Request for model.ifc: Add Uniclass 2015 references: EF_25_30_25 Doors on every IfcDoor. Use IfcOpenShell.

First a look at what the model holds.

```python
import ifcopenshell

model = ifcopenshell.open("model.ifc")
print(model.schema)
print("classifications:", [c.Name for c in model.by_type("IfcClassification")])
for ifc_class in ("IfcDoor", "IfcRoof", "IfcStair", "IfcWall", "IfcWindow"):
    print(ifc_class, len(model.by_type(ifc_class)))
```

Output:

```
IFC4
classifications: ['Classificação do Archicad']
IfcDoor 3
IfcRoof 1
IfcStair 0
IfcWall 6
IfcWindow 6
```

```python
import ifcopenshell
import ifcopenshell.api.classification

model = ifcopenshell.open("model.ifc")

system = ifcopenshell.api.classification.add_classification(model, classification="Uniclass 2015")

codes = {
    "IfcDoor": ("EF_25_30_25", "Doors"),
}
for ifc_class, (code, name) in codes.items():
    products = model.by_type(ifc_class)
    ifcopenshell.api.classification.add_reference(
        model, products=products, classification=system, identification=code, name=name
    )
    print(code, len(products))

model.write("model_rev.ifc")
```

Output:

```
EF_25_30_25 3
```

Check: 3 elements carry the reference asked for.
